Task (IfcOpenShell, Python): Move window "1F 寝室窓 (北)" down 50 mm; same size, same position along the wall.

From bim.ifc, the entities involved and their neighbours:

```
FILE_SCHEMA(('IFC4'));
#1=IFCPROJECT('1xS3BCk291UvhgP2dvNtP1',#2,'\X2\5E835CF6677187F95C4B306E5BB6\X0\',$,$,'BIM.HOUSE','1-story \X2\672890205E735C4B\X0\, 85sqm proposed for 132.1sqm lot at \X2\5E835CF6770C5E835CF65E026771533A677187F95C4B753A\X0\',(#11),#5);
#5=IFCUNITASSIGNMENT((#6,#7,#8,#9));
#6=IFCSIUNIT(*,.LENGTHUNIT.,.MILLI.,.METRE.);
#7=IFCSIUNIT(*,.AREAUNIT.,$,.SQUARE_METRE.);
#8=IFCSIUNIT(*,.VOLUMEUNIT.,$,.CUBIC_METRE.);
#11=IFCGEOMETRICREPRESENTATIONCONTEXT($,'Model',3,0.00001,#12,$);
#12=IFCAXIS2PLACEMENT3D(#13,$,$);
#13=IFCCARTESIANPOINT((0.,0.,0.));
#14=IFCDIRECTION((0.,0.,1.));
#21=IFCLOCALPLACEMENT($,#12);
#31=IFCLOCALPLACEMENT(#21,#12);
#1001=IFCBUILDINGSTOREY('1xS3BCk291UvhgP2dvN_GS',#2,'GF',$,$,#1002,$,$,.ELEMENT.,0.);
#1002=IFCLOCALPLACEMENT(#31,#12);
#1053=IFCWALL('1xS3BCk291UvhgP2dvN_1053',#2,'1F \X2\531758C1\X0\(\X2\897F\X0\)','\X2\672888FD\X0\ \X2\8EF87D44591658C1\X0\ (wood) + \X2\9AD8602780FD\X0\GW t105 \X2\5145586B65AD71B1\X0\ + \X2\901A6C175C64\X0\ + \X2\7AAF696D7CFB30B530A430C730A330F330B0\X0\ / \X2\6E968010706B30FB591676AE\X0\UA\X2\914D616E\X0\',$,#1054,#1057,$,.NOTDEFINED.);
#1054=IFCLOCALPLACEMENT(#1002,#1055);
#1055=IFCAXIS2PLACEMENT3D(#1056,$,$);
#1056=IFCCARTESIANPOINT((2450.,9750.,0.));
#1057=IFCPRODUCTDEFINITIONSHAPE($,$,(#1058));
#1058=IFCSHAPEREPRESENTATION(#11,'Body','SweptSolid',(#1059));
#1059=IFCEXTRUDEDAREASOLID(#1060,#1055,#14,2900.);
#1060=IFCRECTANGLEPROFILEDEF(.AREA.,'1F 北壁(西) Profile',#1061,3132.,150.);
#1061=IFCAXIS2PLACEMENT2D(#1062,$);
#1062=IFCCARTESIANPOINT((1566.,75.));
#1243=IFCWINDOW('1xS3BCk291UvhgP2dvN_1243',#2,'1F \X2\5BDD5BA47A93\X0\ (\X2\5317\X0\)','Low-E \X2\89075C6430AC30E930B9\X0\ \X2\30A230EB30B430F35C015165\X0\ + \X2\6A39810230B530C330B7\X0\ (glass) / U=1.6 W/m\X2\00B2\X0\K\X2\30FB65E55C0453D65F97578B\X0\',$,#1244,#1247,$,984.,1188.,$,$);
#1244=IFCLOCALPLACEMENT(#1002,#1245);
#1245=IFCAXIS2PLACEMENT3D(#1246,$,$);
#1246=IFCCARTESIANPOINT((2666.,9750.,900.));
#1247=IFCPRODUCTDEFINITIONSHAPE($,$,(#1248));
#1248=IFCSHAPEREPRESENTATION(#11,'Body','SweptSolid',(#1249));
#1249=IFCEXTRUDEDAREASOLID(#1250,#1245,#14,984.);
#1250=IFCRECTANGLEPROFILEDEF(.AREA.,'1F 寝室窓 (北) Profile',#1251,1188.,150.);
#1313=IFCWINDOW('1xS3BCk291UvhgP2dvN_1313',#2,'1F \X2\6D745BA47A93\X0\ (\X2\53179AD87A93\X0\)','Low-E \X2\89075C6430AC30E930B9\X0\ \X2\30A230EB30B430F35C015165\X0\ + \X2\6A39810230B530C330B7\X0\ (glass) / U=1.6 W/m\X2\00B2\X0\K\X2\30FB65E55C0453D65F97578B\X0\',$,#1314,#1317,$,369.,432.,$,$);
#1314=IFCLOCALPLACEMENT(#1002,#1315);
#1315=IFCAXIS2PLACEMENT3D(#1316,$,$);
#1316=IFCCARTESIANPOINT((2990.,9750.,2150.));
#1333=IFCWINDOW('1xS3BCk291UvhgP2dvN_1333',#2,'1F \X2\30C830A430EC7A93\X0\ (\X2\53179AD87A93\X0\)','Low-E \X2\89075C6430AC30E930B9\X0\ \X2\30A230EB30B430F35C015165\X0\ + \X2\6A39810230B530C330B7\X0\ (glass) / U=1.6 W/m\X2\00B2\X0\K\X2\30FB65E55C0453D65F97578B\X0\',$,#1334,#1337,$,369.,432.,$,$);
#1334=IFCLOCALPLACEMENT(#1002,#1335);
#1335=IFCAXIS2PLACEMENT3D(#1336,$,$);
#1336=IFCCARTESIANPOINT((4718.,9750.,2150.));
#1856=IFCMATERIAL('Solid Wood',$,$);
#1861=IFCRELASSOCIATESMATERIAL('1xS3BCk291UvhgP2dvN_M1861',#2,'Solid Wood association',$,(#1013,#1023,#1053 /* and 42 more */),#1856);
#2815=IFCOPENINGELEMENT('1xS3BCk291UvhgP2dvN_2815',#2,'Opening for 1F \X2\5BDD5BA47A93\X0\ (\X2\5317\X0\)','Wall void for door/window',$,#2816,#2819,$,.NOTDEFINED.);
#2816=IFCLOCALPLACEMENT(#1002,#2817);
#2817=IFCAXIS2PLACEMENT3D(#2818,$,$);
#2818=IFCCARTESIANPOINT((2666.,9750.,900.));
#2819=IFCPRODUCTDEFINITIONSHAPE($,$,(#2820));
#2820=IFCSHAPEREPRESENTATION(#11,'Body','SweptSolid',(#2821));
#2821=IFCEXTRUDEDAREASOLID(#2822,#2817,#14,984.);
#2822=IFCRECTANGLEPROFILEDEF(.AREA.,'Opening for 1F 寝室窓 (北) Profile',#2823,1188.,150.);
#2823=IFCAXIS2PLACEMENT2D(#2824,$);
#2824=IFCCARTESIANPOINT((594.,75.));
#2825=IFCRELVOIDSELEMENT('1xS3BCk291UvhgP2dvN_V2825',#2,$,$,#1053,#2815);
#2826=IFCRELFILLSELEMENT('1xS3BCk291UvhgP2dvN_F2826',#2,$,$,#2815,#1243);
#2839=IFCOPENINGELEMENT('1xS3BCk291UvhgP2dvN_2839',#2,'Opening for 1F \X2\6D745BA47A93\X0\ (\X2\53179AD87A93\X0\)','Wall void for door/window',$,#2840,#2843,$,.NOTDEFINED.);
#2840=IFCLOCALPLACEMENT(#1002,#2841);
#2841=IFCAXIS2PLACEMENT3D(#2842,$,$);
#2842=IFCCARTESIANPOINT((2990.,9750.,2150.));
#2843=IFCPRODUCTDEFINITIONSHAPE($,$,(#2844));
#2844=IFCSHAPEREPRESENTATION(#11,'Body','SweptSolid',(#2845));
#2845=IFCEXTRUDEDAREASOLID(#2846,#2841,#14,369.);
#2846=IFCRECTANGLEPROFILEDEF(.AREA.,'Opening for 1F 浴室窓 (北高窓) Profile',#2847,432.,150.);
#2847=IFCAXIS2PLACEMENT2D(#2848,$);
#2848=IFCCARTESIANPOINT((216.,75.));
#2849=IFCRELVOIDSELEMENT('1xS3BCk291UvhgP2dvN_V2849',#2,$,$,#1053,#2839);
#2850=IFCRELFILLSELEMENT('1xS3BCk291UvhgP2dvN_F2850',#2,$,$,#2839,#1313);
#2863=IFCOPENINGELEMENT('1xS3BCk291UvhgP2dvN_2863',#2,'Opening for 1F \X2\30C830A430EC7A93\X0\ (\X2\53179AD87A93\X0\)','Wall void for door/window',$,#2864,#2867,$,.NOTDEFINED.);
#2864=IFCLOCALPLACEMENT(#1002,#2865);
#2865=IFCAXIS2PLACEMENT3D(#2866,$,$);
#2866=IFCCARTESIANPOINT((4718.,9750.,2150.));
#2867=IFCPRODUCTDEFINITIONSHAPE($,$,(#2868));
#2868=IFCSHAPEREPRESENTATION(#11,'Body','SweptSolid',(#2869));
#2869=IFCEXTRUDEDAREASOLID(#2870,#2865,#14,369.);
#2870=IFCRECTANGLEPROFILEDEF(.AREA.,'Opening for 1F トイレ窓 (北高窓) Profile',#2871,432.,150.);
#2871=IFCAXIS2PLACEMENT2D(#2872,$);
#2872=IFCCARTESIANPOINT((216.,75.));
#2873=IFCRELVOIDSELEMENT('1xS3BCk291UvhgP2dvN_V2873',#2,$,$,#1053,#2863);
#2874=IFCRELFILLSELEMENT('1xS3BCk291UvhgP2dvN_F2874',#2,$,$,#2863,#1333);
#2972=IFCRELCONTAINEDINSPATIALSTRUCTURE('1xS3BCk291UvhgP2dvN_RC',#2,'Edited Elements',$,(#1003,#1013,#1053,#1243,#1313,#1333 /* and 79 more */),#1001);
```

```python
import numpy as np
import ifcopenshell
import ifcopenshell.api.geometry
import ifcopenshell.util.placement
import ifcopenshell.util.unit

model = ifcopenshell.open("bim.ifc")
unit_scale = ifcopenshell.util.unit.calculate_unit_scale(model)

window = model.by_id(1243)
opening = window.FillsVoids[0].RelatingOpeningElement
dz = -50.0

shift = np.array([0.0, 0.0, dz])
# The window is not placed relative to its opening, so move both.
for product in (opening, window):
    matrix = ifcopenshell.util.placement.get_local_placement(product.ObjectPlacement)
    matrix[:3, 3] += shift
    ifcopenshell.api.geometry.edit_object_placement(model, product=product, matrix=matrix, is_si=False)

print(f"moved by {dz * unit_scale:+.3f} m")

model.write("bim_edited.ifc")
```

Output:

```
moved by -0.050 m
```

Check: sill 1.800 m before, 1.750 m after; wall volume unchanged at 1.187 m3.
